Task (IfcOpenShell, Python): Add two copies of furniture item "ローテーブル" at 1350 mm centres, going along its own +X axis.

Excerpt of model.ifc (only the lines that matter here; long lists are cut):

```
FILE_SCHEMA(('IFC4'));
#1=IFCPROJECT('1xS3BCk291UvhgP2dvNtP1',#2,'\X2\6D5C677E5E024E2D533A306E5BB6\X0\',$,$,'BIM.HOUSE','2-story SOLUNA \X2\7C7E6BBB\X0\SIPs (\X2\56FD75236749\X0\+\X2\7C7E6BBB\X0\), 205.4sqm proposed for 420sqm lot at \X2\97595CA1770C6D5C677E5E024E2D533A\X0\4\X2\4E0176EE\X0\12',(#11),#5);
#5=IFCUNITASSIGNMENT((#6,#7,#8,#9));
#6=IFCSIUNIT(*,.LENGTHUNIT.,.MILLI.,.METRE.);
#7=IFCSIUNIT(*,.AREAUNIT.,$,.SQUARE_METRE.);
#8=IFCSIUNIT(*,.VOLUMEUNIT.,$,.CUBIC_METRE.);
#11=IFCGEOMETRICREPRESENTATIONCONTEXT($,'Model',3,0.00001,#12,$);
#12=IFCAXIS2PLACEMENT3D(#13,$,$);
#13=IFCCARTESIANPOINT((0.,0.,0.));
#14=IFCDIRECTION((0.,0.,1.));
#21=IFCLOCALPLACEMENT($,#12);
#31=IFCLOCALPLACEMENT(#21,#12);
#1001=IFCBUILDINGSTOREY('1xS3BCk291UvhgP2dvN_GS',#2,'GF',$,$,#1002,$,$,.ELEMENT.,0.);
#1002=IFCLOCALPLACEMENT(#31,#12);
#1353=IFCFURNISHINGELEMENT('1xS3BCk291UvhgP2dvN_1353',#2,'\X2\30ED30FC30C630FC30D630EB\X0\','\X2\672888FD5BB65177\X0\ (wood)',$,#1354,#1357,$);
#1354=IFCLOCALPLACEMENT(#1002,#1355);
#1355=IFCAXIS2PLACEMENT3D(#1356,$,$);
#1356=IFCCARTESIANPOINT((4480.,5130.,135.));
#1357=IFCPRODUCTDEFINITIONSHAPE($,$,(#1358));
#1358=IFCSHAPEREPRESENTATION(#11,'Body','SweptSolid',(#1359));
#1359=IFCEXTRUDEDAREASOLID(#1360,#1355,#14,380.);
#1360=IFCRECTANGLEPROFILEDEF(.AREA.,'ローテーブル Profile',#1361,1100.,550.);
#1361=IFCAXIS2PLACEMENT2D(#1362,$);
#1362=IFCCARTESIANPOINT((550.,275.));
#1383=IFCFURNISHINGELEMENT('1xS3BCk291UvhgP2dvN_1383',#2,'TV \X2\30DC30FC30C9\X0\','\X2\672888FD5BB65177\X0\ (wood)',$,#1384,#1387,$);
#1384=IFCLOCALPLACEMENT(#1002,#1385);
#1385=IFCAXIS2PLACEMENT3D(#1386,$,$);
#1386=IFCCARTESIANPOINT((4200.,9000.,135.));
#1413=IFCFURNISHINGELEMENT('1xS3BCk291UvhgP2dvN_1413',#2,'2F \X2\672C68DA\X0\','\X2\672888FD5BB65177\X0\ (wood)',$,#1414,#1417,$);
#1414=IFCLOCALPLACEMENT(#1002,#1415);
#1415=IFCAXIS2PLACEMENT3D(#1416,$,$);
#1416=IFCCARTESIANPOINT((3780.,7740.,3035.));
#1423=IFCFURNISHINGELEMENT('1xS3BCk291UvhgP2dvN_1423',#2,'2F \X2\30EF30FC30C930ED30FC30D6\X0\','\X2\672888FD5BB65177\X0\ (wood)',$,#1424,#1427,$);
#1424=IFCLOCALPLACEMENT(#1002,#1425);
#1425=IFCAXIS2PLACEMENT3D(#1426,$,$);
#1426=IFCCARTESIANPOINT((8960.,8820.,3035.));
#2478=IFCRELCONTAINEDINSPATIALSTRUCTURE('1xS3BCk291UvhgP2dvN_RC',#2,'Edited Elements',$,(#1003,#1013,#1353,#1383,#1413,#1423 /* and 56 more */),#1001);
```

```python
import ifcopenshell
import ifcopenshell.api.geometry
import ifcopenshell.api.root
import ifcopenshell.util.element
import ifcopenshell.util.placement
import ifcopenshell.util.unit

model = ifcopenshell.open("model.ifc")
unit_scale = ifcopenshell.util.unit.calculate_unit_scale(model)


def reuse_history(source, copy):
    """copy_class also copies each property set's owner history, people and application; keep the originals."""
    for rel in copy.IsDefinedBy:
        if rel.is_a("IfcRelDefinesByProperties") and (history := rel.RelatingPropertyDefinition.OwnerHistory):
            rel.RelatingPropertyDefinition.OwnerHistory = source.OwnerHistory
            ifcopenshell.util.element.remove_deep2(model, history)


source = model.by_id(1353)
base = ifcopenshell.util.placement.get_local_placement(source.ObjectPlacement)
step = base[:3, 0] * 1.35 / unit_scale

for i in range(1, 3):
    copy = ifcopenshell.api.root.copy_class(model, product=source)
    copy.Representation = ifcopenshell.util.element.copy_deep(
        model, source.Representation, exclude=["IfcGeometricRepresentationContext", "IfcRepresentationMap"]
    )
    reuse_history(source, copy)
    matrix = base.copy()
    matrix[:3, 3] += i * step
    print("added at", matrix[:3, 3].round(3) + 0.0)
    ifcopenshell.api.geometry.edit_object_placement(model, product=copy, matrix=matrix, is_si=False)

model.write("model_v2.ifc")
```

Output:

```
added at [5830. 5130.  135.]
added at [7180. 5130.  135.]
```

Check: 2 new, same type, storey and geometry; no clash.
